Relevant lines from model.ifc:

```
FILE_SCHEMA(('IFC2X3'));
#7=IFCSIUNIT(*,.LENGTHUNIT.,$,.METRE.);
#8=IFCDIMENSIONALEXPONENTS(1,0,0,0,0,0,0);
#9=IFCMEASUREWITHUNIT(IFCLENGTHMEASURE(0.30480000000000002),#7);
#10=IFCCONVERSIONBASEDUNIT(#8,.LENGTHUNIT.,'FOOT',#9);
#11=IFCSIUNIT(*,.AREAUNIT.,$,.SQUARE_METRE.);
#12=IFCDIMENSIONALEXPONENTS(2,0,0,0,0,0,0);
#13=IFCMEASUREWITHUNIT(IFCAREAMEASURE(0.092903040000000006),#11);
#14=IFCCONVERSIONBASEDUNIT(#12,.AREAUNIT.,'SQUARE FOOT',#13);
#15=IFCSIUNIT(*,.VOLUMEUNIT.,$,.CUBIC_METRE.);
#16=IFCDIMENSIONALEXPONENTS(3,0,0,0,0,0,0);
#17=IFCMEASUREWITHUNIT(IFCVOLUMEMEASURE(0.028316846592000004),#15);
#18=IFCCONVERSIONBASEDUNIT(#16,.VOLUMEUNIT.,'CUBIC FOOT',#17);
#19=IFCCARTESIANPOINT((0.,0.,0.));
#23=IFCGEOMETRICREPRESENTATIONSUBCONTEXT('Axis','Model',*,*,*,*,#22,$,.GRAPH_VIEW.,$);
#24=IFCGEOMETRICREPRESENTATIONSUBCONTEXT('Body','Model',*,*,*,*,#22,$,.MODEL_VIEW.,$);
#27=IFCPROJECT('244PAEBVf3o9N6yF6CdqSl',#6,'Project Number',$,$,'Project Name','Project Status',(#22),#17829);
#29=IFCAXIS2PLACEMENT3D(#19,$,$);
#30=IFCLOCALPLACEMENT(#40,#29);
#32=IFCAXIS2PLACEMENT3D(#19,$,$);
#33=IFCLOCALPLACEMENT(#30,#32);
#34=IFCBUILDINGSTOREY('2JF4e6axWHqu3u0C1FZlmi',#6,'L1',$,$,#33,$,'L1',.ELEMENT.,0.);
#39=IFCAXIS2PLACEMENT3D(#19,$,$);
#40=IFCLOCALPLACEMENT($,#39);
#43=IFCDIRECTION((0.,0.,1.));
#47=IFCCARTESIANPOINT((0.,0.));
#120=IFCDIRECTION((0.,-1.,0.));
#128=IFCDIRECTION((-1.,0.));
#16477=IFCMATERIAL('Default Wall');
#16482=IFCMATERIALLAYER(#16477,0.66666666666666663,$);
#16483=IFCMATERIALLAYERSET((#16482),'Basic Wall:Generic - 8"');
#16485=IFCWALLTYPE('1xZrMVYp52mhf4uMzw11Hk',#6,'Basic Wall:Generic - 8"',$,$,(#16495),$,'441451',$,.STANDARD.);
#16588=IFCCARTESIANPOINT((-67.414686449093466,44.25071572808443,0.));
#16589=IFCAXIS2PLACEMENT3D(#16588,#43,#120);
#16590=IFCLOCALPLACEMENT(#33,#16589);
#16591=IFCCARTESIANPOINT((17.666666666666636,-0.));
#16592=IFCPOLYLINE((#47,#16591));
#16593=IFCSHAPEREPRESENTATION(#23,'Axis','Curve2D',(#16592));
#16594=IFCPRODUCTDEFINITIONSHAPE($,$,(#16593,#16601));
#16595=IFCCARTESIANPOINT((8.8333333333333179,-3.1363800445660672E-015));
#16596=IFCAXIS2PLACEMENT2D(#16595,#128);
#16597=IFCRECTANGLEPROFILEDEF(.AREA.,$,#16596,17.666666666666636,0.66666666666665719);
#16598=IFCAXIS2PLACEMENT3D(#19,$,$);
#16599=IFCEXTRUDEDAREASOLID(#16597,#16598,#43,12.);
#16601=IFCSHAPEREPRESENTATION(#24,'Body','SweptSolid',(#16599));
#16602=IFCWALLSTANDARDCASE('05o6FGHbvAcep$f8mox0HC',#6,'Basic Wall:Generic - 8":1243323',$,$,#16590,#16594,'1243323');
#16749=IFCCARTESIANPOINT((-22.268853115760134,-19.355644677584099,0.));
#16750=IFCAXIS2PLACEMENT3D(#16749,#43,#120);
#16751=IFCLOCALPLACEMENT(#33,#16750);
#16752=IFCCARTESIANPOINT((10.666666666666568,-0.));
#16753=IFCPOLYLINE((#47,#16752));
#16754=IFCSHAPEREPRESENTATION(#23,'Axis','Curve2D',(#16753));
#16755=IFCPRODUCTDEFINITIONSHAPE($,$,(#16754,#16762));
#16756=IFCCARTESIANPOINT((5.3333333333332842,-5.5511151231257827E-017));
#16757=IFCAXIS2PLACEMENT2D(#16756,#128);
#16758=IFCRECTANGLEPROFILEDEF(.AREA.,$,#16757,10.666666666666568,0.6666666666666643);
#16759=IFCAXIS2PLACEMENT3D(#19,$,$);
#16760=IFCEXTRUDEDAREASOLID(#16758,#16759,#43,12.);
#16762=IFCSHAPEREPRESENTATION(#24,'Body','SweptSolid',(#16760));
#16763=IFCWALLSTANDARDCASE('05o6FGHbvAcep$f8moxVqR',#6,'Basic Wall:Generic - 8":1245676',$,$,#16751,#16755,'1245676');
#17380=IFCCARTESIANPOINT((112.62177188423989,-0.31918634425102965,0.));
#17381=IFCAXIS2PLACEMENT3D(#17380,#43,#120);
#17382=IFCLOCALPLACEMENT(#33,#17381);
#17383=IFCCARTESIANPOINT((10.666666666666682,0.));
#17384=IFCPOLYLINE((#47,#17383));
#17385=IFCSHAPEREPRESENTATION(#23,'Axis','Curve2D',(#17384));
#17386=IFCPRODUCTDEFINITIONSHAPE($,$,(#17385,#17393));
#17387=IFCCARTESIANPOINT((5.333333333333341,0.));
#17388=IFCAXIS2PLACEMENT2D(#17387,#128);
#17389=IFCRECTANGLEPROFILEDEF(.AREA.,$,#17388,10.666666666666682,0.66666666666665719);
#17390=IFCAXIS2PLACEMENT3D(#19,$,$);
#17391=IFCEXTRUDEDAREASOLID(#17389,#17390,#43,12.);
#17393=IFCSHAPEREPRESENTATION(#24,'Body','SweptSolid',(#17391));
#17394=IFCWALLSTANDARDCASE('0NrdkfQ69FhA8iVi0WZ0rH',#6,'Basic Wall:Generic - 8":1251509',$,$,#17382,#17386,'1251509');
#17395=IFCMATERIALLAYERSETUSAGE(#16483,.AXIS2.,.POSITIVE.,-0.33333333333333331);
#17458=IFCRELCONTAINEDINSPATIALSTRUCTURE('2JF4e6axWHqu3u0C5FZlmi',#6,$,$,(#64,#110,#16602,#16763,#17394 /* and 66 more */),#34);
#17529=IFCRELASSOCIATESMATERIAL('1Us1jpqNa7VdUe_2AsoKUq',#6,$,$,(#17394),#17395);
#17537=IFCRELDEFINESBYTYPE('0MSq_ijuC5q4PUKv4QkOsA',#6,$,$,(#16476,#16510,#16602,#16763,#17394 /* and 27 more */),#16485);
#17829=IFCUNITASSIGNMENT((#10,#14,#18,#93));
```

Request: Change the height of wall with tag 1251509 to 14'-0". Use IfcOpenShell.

```python
import ifcopenshell
import ifcopenshell.geom
import ifcopenshell.util.representation
import ifcopenshell.util.shape
import ifcopenshell.util.unit

model = ifcopenshell.open("model.ifc")
unit_scale = ifcopenshell.util.unit.calculate_unit_scale(model)
settings = ifcopenshell.geom.settings()


def volume(element):
    """Net volume in cubic metres, openings subtracted."""
    shape = ifcopenshell.geom.create_shape(settings, element)
    return ifcopenshell.util.shape.get_volume(shape.geometry)


wall = model.by_id(17394)
before = volume(wall)

body = ifcopenshell.util.representation.get_representation(wall, "Model", "Body")
solid = body.Items[0]
old_height = solid.Depth
solid.Depth = 168 * 0.0254 / unit_scale
after = volume(wall)

print(f"height {old_height:g} -> {solid.Depth:g}, volume {before:.3f} -> {after:.3f} m3")

model.write("model_rev.ifc")
```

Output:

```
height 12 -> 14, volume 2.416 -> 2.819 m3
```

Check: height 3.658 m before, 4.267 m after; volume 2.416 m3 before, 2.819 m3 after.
